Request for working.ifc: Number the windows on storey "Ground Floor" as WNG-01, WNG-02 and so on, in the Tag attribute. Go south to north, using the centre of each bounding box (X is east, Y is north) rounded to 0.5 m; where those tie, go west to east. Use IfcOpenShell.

First a look at what the model holds.

```python
import ifcopenshell
import ifcopenshell.util.element
import ifcopenshell.util.placement

model = ifcopenshell.open("working.ifc")
print(model.schema)
storey = next(s for s in model.by_type("IfcBuildingStorey") if s.Name == "Ground Floor")
windows = [e for e in ifcopenshell.util.element.get_decomposition(storey) if e.is_a("IfcWindow")]
for e in sorted(windows, key=lambda e: e.id()):
    origin = ifcopenshell.util.placement.get_local_placement(e.ObjectPlacement)[:3, 3]
    print(e.id(), e.Tag, e.Name, origin.round(2) + 0.0, sep=" | ")
```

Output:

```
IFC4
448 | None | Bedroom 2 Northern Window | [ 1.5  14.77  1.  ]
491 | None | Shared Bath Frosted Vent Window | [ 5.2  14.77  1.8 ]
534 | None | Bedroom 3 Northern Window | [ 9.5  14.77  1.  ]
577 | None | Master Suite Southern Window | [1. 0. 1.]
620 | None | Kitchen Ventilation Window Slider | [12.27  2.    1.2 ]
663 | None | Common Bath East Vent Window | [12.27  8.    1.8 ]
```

```python
import ifcopenshell
import ifcopenshell.geom
import ifcopenshell.util.element
import ifcopenshell.util.shape

model = ifcopenshell.open("working.ifc")
settings = ifcopenshell.geom.settings()
settings.set("use-world-coords", True)


def centre(element):
    shape = ifcopenshell.geom.create_shape(settings, element)
    return ifcopenshell.util.shape.get_bbox_centroid(shape.geometry)


storey = next(s for s in model.by_type("IfcBuildingStorey") if s.Name == "Ground Floor")
windows = [e for e in ifcopenshell.util.element.get_decomposition(storey) if e.is_a("IfcWindow")]

# Insertion points can sit at a corner or the storey origin, so sort by the geometry (in metres).
centres = {e: centre(e) for e in windows}
windows.sort(key=lambda e: (round(centres[e][1] / 0.5), centres[e][0]))

for i, e in enumerate(windows, start=1):
    number = f"WNG-{i:02d}"
    e.Tag = number
    print(e.id(), number)

model.write("working_updated.ifc")
```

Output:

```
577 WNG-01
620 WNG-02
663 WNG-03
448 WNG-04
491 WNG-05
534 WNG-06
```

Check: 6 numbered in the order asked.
